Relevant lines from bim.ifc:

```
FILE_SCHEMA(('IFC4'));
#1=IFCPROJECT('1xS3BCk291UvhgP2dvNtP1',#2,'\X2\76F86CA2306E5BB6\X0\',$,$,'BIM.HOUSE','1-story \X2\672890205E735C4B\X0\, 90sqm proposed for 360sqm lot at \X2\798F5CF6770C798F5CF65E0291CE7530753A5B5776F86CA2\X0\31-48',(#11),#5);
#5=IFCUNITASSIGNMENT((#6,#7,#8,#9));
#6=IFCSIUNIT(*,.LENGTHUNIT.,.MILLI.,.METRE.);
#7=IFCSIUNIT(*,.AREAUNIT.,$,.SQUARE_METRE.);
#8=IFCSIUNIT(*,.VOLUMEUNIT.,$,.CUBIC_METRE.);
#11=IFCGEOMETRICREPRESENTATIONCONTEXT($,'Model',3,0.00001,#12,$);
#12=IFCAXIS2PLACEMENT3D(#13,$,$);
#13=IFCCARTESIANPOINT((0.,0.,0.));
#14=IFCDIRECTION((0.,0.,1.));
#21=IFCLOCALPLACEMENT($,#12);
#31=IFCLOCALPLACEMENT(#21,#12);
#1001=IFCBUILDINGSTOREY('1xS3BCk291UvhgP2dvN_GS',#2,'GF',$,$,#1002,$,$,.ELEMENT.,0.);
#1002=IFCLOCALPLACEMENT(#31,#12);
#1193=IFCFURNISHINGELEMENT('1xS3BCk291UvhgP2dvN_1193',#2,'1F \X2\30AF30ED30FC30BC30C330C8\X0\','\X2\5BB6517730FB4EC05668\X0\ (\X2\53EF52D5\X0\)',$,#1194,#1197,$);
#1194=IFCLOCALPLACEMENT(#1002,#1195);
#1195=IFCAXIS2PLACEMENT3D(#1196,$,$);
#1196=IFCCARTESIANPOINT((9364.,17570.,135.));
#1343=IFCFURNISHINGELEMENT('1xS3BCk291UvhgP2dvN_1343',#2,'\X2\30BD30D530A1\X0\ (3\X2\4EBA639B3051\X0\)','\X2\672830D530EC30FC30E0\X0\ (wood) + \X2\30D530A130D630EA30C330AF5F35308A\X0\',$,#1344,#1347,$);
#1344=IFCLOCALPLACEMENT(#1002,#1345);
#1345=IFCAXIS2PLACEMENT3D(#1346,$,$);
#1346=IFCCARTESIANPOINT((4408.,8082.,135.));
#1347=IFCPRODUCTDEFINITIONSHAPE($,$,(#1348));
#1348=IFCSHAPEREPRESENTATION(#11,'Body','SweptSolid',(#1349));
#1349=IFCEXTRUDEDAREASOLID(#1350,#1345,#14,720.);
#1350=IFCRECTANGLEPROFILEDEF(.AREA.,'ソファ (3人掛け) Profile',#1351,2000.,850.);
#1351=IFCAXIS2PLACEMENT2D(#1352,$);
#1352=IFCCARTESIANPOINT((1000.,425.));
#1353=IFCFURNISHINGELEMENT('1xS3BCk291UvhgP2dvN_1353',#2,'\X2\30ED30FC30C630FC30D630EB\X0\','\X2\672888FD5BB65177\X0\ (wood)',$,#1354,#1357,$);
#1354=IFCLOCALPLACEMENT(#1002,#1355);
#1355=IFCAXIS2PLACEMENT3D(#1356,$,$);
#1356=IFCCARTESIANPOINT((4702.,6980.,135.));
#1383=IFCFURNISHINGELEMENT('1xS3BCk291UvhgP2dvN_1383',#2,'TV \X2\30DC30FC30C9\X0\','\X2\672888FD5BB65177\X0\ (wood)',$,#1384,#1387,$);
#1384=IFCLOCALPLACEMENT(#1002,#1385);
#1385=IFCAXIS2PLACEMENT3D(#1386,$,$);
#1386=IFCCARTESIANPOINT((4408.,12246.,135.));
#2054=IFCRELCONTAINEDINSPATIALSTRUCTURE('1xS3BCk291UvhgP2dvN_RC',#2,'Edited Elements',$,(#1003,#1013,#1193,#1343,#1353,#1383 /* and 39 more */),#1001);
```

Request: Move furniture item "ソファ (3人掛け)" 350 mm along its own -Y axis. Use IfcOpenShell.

```python
import ifcopenshell
import ifcopenshell.api.geometry
import ifcopenshell.util.placement

model = ifcopenshell.open("bim.ifc")

item = model.by_id(1343)
matrix = ifcopenshell.util.placement.get_local_placement(item.ObjectPlacement)
matrix[:3, 3] -= matrix[:3, 1] * 350.0
ifcopenshell.api.geometry.edit_object_placement(model, product=item, matrix=matrix, is_si=False)

print(ifcopenshell.util.placement.get_local_placement(item.ObjectPlacement).round(3) + 0.0)

model.write("bim_updated.ifc")
```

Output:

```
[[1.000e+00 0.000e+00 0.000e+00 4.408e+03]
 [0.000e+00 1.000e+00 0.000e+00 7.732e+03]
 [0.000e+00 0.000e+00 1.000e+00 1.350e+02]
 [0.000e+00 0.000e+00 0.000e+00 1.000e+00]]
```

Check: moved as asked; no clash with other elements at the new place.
